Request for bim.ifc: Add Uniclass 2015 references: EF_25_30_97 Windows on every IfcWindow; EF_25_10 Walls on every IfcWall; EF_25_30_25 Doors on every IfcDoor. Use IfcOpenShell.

First a look at what the model holds.

```python
import ifcopenshell

model = ifcopenshell.open("bim.ifc")
print(model.schema)
print("classifications:", [c.Name for c in model.by_type("IfcClassification")])
for ifc_class in ("IfcDoor", "IfcRoof", "IfcStair", "IfcWall", "IfcWindow"):
    print(ifc_class, len(model.by_type(ifc_class)))
```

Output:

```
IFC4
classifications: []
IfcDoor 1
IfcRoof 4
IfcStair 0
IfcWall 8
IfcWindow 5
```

```python
import ifcopenshell
import ifcopenshell.api.classification

model = ifcopenshell.open("bim.ifc")

system = ifcopenshell.api.classification.add_classification(model, classification="Uniclass 2015")

codes = {
    "IfcWindow": ("EF_25_30_97", "Windows"),
    "IfcWall": ("EF_25_10", "Walls"),
    "IfcDoor": ("EF_25_30_25", "Doors"),
}
for ifc_class, (code, name) in codes.items():
    products = model.by_type(ifc_class)
    ifcopenshell.api.classification.add_reference(
        model, products=products, classification=system, identification=code, name=name
    )
    print(code, len(products))

model.write("bim-out.ifc")
```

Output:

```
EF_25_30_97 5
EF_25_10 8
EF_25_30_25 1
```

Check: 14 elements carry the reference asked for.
